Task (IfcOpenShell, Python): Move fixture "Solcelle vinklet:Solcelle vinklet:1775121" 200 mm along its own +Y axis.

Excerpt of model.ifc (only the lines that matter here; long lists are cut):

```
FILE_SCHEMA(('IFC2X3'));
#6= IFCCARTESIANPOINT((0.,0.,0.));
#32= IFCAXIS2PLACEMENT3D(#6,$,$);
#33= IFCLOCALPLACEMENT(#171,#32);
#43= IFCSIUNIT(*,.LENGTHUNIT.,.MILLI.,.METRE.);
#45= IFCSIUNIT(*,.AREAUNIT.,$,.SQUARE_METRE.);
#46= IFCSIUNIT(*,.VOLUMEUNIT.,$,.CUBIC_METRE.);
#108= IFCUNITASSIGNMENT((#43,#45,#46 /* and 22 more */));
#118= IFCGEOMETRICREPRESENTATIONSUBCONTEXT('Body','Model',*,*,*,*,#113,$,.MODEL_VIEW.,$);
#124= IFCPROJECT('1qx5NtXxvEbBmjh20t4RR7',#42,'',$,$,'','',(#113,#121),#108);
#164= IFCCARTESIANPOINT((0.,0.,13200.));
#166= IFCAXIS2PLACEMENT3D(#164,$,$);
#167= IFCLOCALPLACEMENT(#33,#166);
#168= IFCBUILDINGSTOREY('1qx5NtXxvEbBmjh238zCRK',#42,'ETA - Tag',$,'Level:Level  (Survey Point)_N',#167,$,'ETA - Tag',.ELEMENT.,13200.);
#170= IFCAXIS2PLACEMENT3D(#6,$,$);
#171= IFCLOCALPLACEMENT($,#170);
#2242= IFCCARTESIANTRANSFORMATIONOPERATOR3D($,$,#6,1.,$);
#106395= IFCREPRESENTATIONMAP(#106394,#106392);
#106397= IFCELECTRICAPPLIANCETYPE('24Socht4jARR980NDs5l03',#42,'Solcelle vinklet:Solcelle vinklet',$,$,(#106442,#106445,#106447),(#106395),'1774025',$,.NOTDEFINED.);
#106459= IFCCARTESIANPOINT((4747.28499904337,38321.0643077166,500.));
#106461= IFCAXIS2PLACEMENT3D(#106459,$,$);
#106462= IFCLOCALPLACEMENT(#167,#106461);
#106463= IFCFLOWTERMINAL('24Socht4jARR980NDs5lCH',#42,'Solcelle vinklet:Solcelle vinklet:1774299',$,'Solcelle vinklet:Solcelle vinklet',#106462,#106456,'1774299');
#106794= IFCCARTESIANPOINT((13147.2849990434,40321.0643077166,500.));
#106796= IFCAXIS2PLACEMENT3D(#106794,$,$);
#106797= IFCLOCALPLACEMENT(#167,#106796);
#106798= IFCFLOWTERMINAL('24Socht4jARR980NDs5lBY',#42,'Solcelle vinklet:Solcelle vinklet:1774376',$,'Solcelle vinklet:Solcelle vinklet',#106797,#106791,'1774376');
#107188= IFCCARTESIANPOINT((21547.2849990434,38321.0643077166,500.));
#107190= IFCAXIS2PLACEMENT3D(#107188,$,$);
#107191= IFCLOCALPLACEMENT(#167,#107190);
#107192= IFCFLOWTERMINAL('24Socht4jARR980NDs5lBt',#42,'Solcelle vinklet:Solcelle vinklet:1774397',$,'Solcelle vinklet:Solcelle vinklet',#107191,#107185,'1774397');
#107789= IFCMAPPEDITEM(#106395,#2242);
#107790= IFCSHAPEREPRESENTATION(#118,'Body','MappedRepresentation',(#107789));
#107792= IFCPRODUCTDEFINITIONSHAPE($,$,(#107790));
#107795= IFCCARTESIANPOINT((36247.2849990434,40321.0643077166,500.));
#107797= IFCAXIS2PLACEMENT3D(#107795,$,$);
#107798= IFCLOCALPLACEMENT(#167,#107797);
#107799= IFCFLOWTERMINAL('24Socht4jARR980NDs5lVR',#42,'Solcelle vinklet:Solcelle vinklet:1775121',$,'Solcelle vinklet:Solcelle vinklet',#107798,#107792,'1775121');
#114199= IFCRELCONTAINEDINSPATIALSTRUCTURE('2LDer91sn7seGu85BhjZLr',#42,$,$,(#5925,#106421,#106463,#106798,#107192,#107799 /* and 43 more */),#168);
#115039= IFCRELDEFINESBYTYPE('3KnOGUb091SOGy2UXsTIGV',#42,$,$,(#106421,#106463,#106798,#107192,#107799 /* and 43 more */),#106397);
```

```python
import ifcopenshell
import ifcopenshell.api.geometry
import ifcopenshell.util.placement
import ifcopenshell.util.unit

model = ifcopenshell.open("model.ifc")
unit_scale = ifcopenshell.util.unit.calculate_unit_scale(model)

item = model.by_guid("24Socht4jARR980NDs5lVR")
matrix = ifcopenshell.util.placement.get_local_placement(item.ObjectPlacement)
matrix[:3, 3] += matrix[:3, 1] * 0.2 / unit_scale
ifcopenshell.api.geometry.edit_object_placement(model, product=item, matrix=matrix, is_si=False)

print(ifcopenshell.util.placement.get_local_placement(item.ObjectPlacement).round(3) + 0.0)

model.write("model_rev.ifc")
```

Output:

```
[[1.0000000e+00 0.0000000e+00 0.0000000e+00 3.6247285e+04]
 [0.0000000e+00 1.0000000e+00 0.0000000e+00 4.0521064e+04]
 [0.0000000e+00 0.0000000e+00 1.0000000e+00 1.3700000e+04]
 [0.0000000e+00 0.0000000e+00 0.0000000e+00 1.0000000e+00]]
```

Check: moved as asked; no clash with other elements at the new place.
